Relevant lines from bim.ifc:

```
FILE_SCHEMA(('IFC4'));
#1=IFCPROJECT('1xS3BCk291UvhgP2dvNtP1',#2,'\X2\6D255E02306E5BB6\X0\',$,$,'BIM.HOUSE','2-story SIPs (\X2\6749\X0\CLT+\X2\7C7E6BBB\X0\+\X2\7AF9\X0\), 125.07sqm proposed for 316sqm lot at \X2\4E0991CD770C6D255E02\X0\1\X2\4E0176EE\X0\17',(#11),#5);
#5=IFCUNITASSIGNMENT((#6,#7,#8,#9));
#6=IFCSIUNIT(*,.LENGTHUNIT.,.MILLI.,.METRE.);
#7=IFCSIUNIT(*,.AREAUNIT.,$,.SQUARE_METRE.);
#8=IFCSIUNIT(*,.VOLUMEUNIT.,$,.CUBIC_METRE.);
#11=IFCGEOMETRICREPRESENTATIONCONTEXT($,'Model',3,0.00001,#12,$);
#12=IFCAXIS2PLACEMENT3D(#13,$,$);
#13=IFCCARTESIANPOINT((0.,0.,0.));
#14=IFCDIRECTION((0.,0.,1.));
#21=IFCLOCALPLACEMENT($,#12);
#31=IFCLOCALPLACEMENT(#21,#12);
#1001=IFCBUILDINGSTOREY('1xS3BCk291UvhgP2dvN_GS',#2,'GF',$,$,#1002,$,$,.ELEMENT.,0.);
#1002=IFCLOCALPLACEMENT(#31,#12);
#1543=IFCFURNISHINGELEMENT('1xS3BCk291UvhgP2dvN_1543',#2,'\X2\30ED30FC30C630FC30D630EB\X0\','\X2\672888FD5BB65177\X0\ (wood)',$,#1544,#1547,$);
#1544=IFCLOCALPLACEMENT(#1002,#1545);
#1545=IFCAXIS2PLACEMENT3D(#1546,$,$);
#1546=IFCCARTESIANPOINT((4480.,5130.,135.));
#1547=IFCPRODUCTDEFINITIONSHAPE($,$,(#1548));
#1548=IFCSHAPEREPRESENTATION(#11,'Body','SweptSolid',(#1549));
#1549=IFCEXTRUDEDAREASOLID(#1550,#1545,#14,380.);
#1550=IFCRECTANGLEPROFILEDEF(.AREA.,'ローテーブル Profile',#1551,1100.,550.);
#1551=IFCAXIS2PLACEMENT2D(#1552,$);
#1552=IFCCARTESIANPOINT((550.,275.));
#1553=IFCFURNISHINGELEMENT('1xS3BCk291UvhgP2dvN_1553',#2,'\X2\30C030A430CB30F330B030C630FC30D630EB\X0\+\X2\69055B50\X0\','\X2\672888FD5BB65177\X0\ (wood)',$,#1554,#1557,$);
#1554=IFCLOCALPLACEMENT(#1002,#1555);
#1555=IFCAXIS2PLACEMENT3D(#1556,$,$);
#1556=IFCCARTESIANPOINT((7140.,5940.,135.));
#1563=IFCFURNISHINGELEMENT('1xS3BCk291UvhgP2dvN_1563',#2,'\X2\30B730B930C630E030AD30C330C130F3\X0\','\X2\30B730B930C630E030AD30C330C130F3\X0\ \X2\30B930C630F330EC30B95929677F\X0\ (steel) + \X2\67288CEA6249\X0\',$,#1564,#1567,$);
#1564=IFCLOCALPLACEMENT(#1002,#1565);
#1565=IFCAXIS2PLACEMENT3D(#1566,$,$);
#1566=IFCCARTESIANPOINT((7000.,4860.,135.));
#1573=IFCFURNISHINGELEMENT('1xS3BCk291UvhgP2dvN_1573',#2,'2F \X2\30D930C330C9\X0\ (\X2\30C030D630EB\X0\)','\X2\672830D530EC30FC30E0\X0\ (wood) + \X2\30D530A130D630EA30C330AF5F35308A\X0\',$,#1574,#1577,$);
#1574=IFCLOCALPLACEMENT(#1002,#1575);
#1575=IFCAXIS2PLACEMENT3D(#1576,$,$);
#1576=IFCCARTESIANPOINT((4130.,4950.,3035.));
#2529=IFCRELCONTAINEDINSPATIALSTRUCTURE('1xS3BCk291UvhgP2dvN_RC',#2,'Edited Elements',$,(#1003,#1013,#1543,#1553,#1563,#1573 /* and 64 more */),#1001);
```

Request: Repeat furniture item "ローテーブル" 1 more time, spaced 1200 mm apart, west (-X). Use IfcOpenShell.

```python
import numpy as np
import ifcopenshell
import ifcopenshell.api.geometry
import ifcopenshell.api.root
import ifcopenshell.util.element
import ifcopenshell.util.placement
import ifcopenshell.util.unit

model = ifcopenshell.open("bim.ifc")
unit_scale = ifcopenshell.util.unit.calculate_unit_scale(model)


def reuse_history(source, copy):
    """copy_class also copies each property set's owner history, people and application; keep the originals."""
    for rel in copy.IsDefinedBy:
        if rel.is_a("IfcRelDefinesByProperties") and (history := rel.RelatingPropertyDefinition.OwnerHistory):
            rel.RelatingPropertyDefinition.OwnerHistory = source.OwnerHistory
            ifcopenshell.util.element.remove_deep2(model, history)


source = model.by_guid("1xS3BCk291UvhgP2dvN_1543")
base = ifcopenshell.util.placement.get_local_placement(source.ObjectPlacement)
step = np.array([-1.0, 0.0, 0.0]) * 1.2 / unit_scale

for i in range(1, 2):
    copy = ifcopenshell.api.root.copy_class(model, product=source)
    copy.Representation = ifcopenshell.util.element.copy_deep(
        model, source.Representation, exclude=["IfcGeometricRepresentationContext", "IfcRepresentationMap"]
    )
    reuse_history(source, copy)
    matrix = base.copy()
    matrix[:3, 3] += i * step
    print("added at", matrix[:3, 3].round(3) + 0.0)
    ifcopenshell.api.geometry.edit_object_placement(model, product=copy, matrix=matrix, is_si=False)

model.write("bim_edited.ifc")
```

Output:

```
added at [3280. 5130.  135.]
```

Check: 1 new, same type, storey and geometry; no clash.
